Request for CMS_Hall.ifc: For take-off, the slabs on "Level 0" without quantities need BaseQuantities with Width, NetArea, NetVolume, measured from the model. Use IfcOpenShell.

First a look at what the model holds.

```python
import ifcopenshell
import ifcopenshell.util.element
import ifcopenshell.util.unit

model = ifcopenshell.open("CMS_Hall.ifc")
print(model.schema)
for unit_type in ("LENGTHUNIT", "AREAUNIT", "VOLUMEUNIT"):
    print(unit_type, ifcopenshell.util.unit.calculate_unit_scale(model, unit_type))
storey = next(s for s in model.by_type("IfcBuildingStorey") if s.Name == "Level 0")
slabs = [e for e in ifcopenshell.util.element.get_decomposition(storey) if e.is_a("IfcSlab")]
for e in sorted(slabs, key=lambda e: e.id()):
    print(e.id(), e.is_a(), e.Name, list(ifcopenshell.util.element.get_psets(e, qtos_only=True)), sep=" | ")
```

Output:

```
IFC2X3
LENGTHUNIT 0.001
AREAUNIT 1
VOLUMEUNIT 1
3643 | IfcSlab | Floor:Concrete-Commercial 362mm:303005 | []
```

```python
import ifcopenshell
import ifcopenshell.api.pset
import ifcopenshell.geom
import ifcopenshell.util.element
import ifcopenshell.util.shape
import ifcopenshell.util.unit

model = ifcopenshell.open("CMS_Hall.ifc")
unit_scale = ifcopenshell.util.unit.calculate_unit_scale(model)
area_scale = ifcopenshell.util.unit.calculate_unit_scale(model, "AREAUNIT")
volume_scale = ifcopenshell.util.unit.calculate_unit_scale(model, "VOLUMEUNIT")
settings = ifcopenshell.geom.settings()

storey = next(s for s in model.by_type("IfcBuildingStorey") if s.Name == "Level 0")
slabs = [e for e in ifcopenshell.util.element.get_decomposition(storey) if e.is_a("IfcSlab")]

for e in sorted(slabs, key=lambda e: e.id()):
    if ifcopenshell.util.element.get_psets(e, qtos_only=True, should_inherit=False):
        continue
    # Geometry comes back in metres, in the element's own axes.
    shape = ifcopenshell.geom.create_shape(settings, e)
    values = {
        "Width": ifcopenshell.util.shape.get_z(shape.geometry) / unit_scale,
        "NetArea": ifcopenshell.util.shape.get_footprint_area(shape.geometry) / area_scale,
        "NetVolume": ifcopenshell.util.shape.get_volume(shape.geometry) / volume_scale,
    }
    qto = ifcopenshell.api.pset.add_qto(model, product=e, name="BaseQuantities")
    ifcopenshell.api.pset.edit_qto(model, qto=qto, properties=values)
    print(e.id(), {k: round(v, 3) for k, v in values.items()})

model.write("CMS_Hall_updated.ifc")
```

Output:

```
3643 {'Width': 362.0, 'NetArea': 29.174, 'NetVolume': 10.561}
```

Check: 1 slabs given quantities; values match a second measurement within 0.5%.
